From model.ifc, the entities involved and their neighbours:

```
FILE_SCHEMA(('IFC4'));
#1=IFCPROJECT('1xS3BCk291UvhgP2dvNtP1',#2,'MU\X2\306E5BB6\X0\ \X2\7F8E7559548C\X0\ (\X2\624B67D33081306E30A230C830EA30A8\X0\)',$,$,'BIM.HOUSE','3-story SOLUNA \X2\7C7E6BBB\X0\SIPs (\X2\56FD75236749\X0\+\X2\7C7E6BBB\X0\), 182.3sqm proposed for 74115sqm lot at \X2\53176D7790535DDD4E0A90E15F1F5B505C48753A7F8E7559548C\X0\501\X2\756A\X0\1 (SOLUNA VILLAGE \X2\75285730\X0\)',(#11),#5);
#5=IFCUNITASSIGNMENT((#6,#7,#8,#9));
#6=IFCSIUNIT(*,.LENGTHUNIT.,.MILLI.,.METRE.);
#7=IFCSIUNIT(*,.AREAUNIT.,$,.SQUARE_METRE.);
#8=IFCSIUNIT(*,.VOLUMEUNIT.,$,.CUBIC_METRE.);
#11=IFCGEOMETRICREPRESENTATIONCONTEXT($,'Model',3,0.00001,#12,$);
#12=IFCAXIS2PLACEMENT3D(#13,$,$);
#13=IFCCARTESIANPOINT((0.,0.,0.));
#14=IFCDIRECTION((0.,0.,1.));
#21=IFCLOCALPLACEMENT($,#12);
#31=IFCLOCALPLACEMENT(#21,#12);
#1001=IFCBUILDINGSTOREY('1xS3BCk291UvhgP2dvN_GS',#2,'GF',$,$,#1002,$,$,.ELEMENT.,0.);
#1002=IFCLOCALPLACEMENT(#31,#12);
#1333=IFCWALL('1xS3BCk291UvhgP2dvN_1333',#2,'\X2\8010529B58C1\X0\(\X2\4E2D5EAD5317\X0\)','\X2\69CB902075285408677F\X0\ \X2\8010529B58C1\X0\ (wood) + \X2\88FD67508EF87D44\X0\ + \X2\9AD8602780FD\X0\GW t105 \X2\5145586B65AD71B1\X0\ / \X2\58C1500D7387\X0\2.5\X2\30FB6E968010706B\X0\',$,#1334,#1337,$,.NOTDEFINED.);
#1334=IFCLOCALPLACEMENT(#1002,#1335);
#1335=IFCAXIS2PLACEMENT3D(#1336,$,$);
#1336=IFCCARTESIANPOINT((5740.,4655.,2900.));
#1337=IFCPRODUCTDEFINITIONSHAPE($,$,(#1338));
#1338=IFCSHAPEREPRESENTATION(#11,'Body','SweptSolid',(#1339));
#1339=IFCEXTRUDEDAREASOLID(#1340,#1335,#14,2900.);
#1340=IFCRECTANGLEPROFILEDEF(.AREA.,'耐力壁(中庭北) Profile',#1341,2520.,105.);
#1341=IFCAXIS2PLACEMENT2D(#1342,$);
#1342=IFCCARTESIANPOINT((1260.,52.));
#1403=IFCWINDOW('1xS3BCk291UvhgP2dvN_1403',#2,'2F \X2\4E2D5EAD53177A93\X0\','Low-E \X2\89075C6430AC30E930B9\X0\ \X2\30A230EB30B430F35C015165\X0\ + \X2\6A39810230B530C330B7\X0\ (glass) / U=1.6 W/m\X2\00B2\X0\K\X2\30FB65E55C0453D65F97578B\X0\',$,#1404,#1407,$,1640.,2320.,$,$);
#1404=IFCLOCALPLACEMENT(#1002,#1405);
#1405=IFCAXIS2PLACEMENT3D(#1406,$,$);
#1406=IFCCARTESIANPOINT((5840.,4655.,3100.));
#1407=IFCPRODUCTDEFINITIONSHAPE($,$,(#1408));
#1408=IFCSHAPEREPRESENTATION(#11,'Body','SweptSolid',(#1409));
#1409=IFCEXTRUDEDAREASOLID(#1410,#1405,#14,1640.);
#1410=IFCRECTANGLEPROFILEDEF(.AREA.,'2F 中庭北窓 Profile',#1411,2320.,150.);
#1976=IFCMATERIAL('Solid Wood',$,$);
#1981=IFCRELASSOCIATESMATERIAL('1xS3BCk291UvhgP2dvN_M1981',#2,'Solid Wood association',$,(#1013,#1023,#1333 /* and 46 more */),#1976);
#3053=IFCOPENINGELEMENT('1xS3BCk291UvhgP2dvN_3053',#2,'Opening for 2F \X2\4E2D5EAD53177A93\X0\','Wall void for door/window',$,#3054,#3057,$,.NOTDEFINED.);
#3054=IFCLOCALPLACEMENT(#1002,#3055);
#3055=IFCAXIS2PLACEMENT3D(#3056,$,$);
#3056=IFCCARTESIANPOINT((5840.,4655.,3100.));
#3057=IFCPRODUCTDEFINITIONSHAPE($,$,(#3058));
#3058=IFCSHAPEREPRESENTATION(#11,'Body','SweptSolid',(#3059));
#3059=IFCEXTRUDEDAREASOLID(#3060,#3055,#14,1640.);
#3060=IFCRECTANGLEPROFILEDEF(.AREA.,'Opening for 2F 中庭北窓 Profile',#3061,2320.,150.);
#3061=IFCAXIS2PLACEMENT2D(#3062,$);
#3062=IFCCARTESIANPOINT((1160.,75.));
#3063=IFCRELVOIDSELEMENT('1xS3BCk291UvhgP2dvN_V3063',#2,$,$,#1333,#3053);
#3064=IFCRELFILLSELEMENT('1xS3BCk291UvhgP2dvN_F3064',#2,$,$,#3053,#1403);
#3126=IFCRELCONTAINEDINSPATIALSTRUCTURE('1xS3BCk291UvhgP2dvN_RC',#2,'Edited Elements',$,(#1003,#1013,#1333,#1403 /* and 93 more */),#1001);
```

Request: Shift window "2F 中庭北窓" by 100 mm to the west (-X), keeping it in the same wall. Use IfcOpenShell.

```python
import ifcopenshell
import ifcopenshell.api.geometry
import ifcopenshell.util.placement

model = ifcopenshell.open("model.ifc")

window = model.by_guid("1xS3BCk291UvhgP2dvN_1403")
opening = window.FillsVoids[0].RelatingOpeningElement
wall = opening.VoidsElements[0].RelatingBuildingElement

wall_matrix = ifcopenshell.util.placement.get_local_placement(wall.ObjectPlacement)
shift = wall_matrix[:3, 0] * -100.0
before = ifcopenshell.util.placement.get_local_placement(window.ObjectPlacement)[:3, 3].copy()

# The window is not placed relative to its opening, so move both.
for product in (opening, window):
    matrix = ifcopenshell.util.placement.get_local_placement(product.ObjectPlacement)
    matrix[:3, 3] += shift
    ifcopenshell.api.geometry.edit_object_placement(model, product=product, matrix=matrix, is_si=False)

after = ifcopenshell.util.placement.get_local_placement(window.ObjectPlacement)[:3, 3]
print("window moved by", (after - before).round(3) + 0.0)

model.write("model_v2.ifc")
```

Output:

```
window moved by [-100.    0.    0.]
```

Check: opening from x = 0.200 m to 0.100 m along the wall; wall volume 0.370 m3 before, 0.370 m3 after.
